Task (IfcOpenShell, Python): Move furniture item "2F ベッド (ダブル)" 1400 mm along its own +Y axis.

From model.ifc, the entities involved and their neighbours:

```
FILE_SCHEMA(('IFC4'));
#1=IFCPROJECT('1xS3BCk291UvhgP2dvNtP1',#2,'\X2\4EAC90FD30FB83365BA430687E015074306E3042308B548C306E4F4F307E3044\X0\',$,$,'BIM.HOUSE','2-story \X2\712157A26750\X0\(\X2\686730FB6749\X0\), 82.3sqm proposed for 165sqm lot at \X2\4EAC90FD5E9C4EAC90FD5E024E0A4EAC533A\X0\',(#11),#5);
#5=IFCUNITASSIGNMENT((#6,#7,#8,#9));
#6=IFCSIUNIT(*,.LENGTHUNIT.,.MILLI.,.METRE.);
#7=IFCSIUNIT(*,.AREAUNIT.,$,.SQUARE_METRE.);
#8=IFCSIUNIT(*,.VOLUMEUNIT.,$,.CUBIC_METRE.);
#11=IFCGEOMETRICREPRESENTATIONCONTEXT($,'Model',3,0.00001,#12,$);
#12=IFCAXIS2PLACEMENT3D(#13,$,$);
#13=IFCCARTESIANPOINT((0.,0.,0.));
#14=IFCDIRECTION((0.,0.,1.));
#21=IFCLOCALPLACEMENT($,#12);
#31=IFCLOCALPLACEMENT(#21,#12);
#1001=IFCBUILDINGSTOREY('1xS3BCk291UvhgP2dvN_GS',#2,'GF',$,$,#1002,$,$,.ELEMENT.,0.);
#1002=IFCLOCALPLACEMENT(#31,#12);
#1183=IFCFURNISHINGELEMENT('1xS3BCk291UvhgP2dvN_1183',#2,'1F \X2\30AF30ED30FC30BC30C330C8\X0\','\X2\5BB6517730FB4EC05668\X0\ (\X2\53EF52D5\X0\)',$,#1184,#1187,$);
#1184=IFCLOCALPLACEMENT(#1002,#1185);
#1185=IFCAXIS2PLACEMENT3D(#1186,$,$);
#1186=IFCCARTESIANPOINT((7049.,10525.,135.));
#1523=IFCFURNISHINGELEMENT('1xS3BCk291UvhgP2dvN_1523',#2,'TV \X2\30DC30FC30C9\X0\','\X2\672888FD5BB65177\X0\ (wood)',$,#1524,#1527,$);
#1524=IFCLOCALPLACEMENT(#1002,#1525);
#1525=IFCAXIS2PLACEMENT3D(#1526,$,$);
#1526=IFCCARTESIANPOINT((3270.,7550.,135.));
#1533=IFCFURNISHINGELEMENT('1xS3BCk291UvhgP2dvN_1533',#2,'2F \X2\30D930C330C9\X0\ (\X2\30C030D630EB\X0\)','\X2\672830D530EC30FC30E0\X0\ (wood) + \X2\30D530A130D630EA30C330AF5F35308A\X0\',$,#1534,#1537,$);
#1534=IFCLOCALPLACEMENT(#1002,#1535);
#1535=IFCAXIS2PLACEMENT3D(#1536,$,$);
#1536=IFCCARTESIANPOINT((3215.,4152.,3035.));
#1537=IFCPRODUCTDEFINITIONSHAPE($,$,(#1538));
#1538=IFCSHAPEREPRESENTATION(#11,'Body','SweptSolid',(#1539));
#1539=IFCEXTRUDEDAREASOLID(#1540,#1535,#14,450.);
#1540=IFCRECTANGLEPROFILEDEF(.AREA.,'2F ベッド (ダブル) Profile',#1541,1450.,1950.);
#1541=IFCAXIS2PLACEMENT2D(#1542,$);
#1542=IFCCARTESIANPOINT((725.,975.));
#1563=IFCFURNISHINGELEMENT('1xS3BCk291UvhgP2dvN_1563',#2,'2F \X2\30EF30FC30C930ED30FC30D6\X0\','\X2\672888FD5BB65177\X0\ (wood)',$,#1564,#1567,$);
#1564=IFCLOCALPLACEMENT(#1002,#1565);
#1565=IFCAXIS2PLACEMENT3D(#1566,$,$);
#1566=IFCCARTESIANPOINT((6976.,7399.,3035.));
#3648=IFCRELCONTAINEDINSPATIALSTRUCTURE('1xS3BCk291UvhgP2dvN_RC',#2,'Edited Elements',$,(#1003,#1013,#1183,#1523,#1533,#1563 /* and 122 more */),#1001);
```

```python
import ifcopenshell
import ifcopenshell.api.geometry
import ifcopenshell.util.placement
import ifcopenshell.util.unit

model = ifcopenshell.open("model.ifc")
unit_scale = ifcopenshell.util.unit.calculate_unit_scale(model)

item = model.by_id(1533)
matrix = ifcopenshell.util.placement.get_local_placement(item.ObjectPlacement)
matrix[:3, 3] += matrix[:3, 1] * 1.4 / unit_scale
ifcopenshell.api.geometry.edit_object_placement(model, product=item, matrix=matrix, is_si=False)

print(ifcopenshell.util.placement.get_local_placement(item.ObjectPlacement).round(3) + 0.0)

model.write("model_v2.ifc")
```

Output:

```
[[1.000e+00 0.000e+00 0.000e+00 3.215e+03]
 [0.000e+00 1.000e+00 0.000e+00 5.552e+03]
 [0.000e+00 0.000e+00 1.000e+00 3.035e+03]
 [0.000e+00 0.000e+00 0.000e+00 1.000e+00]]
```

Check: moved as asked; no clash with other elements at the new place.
